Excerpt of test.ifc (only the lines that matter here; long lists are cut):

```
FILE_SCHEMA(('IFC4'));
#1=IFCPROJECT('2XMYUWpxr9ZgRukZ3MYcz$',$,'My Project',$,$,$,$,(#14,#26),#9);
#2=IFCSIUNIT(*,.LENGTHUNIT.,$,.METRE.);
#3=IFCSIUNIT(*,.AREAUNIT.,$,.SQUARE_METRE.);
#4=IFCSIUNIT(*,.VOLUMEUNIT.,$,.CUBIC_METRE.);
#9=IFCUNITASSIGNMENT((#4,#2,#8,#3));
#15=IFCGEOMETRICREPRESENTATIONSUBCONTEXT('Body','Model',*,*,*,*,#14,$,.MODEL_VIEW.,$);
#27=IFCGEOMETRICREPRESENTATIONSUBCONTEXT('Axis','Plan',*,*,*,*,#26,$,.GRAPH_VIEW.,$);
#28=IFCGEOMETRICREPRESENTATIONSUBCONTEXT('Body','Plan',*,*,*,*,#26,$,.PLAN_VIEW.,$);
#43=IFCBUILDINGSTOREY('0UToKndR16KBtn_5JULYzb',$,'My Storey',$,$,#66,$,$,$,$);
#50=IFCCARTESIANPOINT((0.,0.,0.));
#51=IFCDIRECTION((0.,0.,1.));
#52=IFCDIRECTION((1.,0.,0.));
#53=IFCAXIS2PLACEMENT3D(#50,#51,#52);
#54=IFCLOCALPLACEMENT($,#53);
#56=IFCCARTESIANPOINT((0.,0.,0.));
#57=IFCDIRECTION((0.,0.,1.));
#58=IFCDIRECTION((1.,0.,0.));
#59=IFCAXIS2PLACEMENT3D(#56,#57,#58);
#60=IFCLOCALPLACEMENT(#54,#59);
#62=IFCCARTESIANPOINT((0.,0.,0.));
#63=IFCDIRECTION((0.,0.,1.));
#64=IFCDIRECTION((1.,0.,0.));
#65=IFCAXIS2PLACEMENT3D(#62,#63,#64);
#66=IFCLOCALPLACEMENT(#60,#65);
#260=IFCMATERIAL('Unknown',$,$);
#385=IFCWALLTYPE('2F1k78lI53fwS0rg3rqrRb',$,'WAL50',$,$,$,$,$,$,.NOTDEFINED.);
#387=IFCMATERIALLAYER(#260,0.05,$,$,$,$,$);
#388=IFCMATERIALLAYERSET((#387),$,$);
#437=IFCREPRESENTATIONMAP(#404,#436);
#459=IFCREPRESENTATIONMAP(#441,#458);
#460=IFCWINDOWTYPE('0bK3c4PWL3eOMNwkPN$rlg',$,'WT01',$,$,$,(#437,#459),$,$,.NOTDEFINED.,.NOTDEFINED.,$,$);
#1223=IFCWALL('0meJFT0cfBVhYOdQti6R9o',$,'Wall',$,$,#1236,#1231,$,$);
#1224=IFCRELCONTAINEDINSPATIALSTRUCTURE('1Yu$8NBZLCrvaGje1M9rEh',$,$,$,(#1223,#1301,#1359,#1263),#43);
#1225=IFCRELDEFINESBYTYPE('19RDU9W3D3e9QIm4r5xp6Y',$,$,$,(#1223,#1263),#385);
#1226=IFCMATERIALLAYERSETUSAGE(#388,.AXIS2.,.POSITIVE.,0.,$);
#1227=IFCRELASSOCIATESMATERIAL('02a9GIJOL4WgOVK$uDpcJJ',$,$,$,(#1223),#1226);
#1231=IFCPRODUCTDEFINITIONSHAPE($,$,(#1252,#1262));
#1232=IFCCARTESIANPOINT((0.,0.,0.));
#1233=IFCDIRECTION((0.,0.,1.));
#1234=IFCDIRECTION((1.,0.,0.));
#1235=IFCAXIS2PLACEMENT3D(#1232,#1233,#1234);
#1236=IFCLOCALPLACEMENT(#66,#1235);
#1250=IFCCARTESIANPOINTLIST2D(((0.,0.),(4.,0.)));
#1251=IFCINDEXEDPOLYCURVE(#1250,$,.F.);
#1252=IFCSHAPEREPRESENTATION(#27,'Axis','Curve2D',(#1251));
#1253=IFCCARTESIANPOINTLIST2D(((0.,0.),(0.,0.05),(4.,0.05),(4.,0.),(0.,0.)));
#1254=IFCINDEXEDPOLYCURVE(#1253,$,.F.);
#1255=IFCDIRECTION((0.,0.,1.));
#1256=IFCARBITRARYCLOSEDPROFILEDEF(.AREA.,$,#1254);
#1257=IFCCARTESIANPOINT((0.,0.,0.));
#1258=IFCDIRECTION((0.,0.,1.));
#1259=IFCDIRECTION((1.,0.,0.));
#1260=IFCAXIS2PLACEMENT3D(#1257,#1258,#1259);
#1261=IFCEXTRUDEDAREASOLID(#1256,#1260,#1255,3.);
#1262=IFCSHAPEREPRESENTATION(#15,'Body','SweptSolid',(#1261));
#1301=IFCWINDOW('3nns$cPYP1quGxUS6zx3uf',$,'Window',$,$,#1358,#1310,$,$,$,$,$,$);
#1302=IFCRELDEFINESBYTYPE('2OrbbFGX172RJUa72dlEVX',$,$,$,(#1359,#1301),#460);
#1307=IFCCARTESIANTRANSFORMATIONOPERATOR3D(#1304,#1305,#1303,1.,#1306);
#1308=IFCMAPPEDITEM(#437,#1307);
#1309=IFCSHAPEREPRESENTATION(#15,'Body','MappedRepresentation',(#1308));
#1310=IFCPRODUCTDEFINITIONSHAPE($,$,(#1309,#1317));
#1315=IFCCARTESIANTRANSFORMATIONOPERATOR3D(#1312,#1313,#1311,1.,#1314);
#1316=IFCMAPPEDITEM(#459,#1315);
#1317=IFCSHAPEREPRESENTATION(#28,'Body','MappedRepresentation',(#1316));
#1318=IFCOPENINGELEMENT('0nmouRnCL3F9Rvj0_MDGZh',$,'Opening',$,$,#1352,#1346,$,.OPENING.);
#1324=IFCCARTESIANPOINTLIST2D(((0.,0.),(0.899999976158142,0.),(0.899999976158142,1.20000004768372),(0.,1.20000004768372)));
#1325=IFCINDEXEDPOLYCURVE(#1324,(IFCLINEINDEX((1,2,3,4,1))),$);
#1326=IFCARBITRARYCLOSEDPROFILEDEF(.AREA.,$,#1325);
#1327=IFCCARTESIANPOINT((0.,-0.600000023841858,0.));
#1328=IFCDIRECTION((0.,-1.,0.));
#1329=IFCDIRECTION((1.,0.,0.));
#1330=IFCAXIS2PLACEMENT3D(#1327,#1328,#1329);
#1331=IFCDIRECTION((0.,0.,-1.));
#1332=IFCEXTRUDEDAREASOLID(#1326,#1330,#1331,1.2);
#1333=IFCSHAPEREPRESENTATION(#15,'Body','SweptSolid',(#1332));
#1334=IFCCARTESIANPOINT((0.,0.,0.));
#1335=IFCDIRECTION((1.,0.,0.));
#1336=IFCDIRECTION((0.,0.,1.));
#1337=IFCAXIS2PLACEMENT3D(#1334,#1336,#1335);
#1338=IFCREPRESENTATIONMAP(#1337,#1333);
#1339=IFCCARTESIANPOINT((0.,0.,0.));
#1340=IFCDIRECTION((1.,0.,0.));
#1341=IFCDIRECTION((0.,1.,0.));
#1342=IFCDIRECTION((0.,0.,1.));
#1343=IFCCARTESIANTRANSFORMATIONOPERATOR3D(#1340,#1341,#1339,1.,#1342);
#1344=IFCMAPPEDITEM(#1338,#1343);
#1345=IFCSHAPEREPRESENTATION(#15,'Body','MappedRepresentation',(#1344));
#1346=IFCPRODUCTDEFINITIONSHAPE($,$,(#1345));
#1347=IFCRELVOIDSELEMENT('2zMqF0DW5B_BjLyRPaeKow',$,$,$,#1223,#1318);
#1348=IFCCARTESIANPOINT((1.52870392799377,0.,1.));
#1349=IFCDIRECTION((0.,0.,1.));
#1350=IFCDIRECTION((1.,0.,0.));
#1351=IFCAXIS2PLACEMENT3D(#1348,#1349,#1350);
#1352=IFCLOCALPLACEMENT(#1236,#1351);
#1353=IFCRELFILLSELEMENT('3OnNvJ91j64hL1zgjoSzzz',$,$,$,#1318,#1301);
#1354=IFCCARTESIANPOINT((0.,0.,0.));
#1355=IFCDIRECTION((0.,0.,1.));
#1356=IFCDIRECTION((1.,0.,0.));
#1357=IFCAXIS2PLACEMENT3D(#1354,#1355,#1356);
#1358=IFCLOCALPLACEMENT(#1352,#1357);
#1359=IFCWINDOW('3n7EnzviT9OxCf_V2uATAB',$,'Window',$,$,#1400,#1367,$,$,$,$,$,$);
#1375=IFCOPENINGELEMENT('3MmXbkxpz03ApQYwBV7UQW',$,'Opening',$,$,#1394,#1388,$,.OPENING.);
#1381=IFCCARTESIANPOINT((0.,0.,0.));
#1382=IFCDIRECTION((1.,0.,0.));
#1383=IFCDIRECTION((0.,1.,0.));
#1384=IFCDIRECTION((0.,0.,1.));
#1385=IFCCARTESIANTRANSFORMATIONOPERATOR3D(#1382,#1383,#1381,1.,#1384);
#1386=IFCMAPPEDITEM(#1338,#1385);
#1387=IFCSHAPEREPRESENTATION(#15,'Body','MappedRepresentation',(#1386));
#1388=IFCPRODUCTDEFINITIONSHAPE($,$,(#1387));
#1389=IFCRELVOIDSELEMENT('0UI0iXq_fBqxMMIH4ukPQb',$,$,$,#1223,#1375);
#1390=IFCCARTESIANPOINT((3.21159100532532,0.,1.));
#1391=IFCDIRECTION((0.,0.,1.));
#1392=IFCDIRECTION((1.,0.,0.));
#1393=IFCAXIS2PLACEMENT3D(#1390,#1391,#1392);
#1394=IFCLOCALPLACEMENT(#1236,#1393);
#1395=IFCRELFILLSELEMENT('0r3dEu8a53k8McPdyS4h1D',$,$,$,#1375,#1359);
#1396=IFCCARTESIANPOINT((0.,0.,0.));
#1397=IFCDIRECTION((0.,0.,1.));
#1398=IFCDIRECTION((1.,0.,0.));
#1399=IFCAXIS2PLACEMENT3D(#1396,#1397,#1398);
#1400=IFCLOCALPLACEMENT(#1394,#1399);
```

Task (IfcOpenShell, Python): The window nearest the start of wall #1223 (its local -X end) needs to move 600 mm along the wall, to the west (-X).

```python
import ifcopenshell
import ifcopenshell.api.geometry
import ifcopenshell.util.placement

model = ifcopenshell.open("test.ifc")

window = model.by_guid("3nns$cPYP1quGxUS6zx3uf")
opening = window.FillsVoids[0].RelatingOpeningElement
wall = opening.VoidsElements[0].RelatingBuildingElement

wall_matrix = ifcopenshell.util.placement.get_local_placement(wall.ObjectPlacement)
shift = wall_matrix[:3, 0] * -0.6
before = ifcopenshell.util.placement.get_local_placement(window.ObjectPlacement)[:3, 3].copy()

# The window is placed relative to its opening, so it follows when the opening moves.
matrix = ifcopenshell.util.placement.get_local_placement(opening.ObjectPlacement)
matrix[:3, 3] += shift
ifcopenshell.api.geometry.edit_object_placement(
    model, product=opening, matrix=matrix, is_si=False, should_transform_children=True
)

after = ifcopenshell.util.placement.get_local_placement(window.ObjectPlacement)[:3, 3]
print("window moved by", (after - before).round(3) + 0.0)

model.write("test_updated.ifc")
```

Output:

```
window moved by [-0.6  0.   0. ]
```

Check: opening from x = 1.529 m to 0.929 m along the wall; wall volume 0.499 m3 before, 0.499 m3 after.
